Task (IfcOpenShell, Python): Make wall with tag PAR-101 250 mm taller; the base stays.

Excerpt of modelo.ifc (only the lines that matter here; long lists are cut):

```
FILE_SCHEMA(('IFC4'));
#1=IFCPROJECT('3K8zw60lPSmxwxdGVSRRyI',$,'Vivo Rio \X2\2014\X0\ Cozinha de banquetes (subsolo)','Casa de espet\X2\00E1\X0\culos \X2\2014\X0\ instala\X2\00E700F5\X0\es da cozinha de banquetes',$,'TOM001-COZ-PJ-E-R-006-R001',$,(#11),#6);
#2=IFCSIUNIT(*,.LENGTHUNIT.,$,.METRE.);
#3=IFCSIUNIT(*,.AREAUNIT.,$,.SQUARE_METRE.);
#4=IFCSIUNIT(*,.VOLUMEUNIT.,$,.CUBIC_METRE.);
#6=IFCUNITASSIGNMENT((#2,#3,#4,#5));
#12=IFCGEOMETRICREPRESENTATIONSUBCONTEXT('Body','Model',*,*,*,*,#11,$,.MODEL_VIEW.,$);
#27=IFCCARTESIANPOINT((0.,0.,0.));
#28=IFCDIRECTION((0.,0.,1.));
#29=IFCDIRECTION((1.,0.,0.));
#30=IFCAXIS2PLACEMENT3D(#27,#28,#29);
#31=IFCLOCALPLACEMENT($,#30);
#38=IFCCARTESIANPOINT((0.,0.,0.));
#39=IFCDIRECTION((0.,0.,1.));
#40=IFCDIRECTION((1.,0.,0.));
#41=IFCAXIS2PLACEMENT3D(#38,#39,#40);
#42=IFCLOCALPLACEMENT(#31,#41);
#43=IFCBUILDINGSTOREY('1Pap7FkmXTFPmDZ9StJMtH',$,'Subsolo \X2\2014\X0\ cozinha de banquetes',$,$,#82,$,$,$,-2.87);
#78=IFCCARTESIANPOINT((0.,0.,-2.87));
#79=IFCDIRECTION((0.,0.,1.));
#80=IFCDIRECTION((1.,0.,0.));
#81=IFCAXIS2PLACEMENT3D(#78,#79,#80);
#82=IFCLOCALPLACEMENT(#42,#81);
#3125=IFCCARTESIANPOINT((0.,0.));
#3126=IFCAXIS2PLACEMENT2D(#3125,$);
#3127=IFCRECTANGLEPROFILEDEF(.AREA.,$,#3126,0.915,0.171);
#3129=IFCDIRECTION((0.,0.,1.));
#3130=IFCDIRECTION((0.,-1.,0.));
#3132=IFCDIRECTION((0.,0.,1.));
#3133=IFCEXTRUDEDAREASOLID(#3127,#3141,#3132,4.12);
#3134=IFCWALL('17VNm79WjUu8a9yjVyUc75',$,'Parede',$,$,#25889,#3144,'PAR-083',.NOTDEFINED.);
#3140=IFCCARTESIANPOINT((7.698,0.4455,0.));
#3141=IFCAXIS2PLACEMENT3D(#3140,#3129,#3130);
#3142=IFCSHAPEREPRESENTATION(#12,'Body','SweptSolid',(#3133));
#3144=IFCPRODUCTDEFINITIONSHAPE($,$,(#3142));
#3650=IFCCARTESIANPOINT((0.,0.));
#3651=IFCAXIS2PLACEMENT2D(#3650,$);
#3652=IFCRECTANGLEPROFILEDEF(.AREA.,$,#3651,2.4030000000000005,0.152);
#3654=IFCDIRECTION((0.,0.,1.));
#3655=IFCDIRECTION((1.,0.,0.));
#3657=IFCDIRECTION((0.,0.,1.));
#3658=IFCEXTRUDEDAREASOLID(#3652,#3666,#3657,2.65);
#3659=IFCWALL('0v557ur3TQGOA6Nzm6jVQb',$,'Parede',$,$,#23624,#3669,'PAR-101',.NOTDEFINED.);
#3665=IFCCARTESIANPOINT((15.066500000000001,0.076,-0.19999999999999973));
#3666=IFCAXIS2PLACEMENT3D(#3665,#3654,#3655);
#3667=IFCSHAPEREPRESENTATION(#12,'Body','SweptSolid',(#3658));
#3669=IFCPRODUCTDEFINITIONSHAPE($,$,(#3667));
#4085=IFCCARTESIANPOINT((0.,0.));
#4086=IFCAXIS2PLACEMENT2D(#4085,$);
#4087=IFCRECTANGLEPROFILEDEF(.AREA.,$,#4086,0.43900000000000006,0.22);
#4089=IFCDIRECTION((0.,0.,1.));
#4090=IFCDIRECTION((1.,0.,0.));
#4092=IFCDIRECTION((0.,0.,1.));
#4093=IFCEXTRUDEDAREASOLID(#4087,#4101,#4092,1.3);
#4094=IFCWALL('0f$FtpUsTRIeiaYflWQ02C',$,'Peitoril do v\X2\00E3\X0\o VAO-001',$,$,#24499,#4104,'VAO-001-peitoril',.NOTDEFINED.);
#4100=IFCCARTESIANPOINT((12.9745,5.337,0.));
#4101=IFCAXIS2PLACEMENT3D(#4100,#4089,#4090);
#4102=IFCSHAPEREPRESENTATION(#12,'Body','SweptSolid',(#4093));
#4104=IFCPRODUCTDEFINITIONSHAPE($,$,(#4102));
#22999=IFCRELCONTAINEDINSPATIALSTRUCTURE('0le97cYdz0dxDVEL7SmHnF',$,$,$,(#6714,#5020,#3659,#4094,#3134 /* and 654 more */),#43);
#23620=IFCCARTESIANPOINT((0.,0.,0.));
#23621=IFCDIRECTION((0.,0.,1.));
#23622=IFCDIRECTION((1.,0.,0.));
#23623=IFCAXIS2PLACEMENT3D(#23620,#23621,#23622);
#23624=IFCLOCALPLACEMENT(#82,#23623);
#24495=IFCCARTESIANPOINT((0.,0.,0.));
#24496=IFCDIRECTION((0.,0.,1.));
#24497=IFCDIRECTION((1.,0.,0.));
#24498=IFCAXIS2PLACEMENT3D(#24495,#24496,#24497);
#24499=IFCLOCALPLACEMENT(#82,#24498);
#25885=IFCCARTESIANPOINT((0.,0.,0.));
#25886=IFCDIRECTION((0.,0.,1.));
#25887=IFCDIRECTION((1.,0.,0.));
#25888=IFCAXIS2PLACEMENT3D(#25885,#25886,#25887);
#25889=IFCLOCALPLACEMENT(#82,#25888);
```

```python
import ifcopenshell
import ifcopenshell.geom
import ifcopenshell.util.representation
import ifcopenshell.util.shape
import ifcopenshell.util.unit

model = ifcopenshell.open("modelo.ifc")
unit_scale = ifcopenshell.util.unit.calculate_unit_scale(model)
settings = ifcopenshell.geom.settings()


def volume(element):
    """Net volume in cubic metres, openings subtracted."""
    shape = ifcopenshell.geom.create_shape(settings, element)
    return ifcopenshell.util.shape.get_volume(shape.geometry)


wall = model.by_id(3659)
before = volume(wall)

body = ifcopenshell.util.representation.get_representation(wall, "Model", "Body")
solid = body.Items[0]
old_height = solid.Depth
solid.Depth += 0.25 / unit_scale
after = volume(wall)

print(f"height {old_height:g} -> {solid.Depth:g}, volume {before:.3f} -> {after:.3f} m3")

model.write("modelo-out.ifc")
```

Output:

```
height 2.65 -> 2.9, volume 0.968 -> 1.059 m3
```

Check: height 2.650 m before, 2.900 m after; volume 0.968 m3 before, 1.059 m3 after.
